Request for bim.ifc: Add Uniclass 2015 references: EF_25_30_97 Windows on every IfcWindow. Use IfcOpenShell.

First a look at what the model holds.

```python
import ifcopenshell

model = ifcopenshell.open("bim.ifc")
print(model.schema)
print("classifications:", [c.Name for c in model.by_type("IfcClassification")])
for ifc_class in ("IfcDoor", "IfcRoof", "IfcStair", "IfcWall", "IfcWindow"):
    print(ifc_class, len(model.by_type(ifc_class)))
```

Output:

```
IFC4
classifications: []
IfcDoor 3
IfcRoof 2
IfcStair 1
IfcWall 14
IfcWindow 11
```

```python
import ifcopenshell
import ifcopenshell.api.classification

model = ifcopenshell.open("bim.ifc")

system = ifcopenshell.api.classification.add_classification(model, classification="Uniclass 2015")

codes = {
    "IfcWindow": ("EF_25_30_97", "Windows"),
}
for ifc_class, (code, name) in codes.items():
    products = model.by_type(ifc_class)
    ifcopenshell.api.classification.add_reference(
        model, products=products, classification=system, identification=code, name=name
    )
    print(code, len(products))

model.write("bim_updated.ifc")
```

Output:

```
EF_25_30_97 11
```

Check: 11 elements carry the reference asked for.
